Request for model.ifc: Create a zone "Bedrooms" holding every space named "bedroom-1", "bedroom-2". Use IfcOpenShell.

First a look at what the model holds.

```python
import ifcopenshell

model = ifcopenshell.open("model.ifc")
print(model.schema)
seen = {}
for space in model.by_type("IfcSpace"):
    seen[space.Name] = seen.get(space.Name, 0) + 1
for name, count in sorted(seen.items(), key=str):
    print(count, "x", name)
print("zones:", [z.Name for z in model.by_type("IfcZone")][:20])
```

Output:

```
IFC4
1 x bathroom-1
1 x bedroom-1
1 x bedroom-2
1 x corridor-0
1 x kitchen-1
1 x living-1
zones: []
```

```python
import ifcopenshell
import ifcopenshell.api.group
import ifcopenshell.api.root

model = ifcopenshell.open("model.ifc")

names = {"bedroom-1", "bedroom-2"}
spaces = [s for s in model.by_type("IfcSpace") if s.Name in names]

zone = ifcopenshell.api.root.create_entity(model, ifc_class="IfcZone", name="Bedrooms")
ifcopenshell.api.group.assign_group(model, products=spaces, group=zone)
print(len(spaces), "spaces in", zone.Name)

model.write("model_v2.ifc")
```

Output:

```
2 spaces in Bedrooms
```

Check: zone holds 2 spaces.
